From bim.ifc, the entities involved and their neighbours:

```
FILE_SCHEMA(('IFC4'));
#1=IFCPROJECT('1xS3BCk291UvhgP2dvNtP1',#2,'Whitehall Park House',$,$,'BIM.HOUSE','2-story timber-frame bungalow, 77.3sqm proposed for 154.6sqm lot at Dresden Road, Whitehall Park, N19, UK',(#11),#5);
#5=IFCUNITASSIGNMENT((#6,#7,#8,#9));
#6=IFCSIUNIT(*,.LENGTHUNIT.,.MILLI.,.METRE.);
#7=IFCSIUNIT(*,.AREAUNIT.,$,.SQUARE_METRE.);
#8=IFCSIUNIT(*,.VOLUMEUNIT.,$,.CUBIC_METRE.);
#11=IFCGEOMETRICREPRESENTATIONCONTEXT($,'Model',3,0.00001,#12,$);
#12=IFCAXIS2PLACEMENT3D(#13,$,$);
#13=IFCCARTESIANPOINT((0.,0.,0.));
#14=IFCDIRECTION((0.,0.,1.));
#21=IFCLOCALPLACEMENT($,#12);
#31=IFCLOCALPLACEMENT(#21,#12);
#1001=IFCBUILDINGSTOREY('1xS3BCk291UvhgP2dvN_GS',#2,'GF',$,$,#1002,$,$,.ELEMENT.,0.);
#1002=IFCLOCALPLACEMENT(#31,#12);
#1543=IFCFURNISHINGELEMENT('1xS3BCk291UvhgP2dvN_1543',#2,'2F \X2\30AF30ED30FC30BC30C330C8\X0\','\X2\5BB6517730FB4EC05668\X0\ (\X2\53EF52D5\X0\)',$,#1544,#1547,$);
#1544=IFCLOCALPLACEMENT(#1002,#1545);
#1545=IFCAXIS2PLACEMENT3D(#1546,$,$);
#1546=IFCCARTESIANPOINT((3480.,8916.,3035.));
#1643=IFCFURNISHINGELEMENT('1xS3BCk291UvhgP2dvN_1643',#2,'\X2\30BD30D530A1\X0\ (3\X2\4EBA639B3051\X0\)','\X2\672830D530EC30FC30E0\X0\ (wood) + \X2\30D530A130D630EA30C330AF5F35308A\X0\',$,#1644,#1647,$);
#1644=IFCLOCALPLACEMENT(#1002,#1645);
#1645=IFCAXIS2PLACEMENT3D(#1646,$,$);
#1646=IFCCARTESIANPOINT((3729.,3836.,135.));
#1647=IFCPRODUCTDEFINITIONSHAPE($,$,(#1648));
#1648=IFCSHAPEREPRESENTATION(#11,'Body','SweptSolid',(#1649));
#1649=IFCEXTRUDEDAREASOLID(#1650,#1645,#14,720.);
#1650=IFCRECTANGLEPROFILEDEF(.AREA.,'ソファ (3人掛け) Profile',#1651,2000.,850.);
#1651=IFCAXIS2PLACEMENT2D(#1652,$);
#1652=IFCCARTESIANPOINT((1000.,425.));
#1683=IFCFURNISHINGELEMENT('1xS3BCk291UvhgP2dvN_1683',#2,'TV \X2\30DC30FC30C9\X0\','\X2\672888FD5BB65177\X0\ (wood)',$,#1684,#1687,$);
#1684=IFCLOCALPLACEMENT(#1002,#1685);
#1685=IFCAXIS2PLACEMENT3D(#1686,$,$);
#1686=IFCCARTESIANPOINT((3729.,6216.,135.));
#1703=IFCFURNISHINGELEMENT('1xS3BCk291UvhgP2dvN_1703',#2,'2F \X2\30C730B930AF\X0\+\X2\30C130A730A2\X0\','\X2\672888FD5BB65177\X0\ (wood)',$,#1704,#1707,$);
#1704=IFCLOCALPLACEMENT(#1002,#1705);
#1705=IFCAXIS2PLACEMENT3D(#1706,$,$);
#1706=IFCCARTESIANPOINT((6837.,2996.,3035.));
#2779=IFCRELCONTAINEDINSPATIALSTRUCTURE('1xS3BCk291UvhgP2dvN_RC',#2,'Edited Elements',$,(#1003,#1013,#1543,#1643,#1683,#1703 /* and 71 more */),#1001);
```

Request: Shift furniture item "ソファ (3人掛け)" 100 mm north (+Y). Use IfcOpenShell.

```python
import ifcopenshell
import ifcopenshell.api.geometry
import ifcopenshell.util.placement
import ifcopenshell.util.unit

model = ifcopenshell.open("bim.ifc")
unit_scale = ifcopenshell.util.unit.calculate_unit_scale(model)

item = model.by_guid("1xS3BCk291UvhgP2dvN_1643")
matrix = ifcopenshell.util.placement.get_local_placement(item.ObjectPlacement)
matrix[1, 3] += 0.1 / unit_scale
ifcopenshell.api.geometry.edit_object_placement(model, product=item, matrix=matrix, is_si=False)

print(ifcopenshell.util.placement.get_local_placement(item.ObjectPlacement).round(3) + 0.0)

model.write("bim_v2.ifc")
```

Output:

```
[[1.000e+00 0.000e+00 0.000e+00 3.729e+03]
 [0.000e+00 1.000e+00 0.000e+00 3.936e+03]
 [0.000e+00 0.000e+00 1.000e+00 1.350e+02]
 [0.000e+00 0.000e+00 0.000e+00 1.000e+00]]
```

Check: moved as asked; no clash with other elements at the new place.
